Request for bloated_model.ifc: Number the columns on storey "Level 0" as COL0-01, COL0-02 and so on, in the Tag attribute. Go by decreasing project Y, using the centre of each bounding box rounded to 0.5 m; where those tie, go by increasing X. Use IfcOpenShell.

First a look at what the model holds.

```python
import ifcopenshell
import ifcopenshell.util.element
import ifcopenshell.util.placement

model = ifcopenshell.open("bloated_model.ifc")
print(model.schema)
storey = next(s for s in model.by_type("IfcBuildingStorey") if s.Name == "Level 0")
columns = [e for e in ifcopenshell.util.element.get_decomposition(storey) if e.is_a("IfcColumn")]
for e in sorted(columns, key=lambda e: e.id()):
    origin = ifcopenshell.util.placement.get_local_placement(e.ObjectPlacement)[:3, 3]
    print(e.id(), e.Tag, e.Name, origin.round(2) + 0.0, sep=" | ")
```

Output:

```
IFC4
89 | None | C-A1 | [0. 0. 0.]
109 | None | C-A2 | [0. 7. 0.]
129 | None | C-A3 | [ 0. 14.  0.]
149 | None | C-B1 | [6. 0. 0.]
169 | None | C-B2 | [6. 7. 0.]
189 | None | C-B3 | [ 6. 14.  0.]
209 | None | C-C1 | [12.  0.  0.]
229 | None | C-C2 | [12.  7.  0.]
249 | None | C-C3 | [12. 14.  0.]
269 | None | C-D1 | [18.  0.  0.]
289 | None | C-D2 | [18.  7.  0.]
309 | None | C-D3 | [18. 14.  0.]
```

```python
import ifcopenshell
import ifcopenshell.geom
import ifcopenshell.util.element
import ifcopenshell.util.shape

model = ifcopenshell.open("bloated_model.ifc")
settings = ifcopenshell.geom.settings()
settings.set("use-world-coords", True)


def centre(element):
    shape = ifcopenshell.geom.create_shape(settings, element)
    return ifcopenshell.util.shape.get_bbox_centroid(shape.geometry)


storey = next(s for s in model.by_type("IfcBuildingStorey") if s.Name == "Level 0")
columns = [e for e in ifcopenshell.util.element.get_decomposition(storey) if e.is_a("IfcColumn")]

# Insertion points can sit at a corner or the storey origin, so sort by the geometry (in metres).
centres = {e: centre(e) for e in columns}
columns.sort(key=lambda e: (-round(centres[e][1] / 0.5), centres[e][0]))

for i, e in enumerate(columns, start=1):
    number = f"COL0-{i:02d}"
    e.Tag = number
    print(e.id(), number)

model.write("bloated_model_edited.ifc")
```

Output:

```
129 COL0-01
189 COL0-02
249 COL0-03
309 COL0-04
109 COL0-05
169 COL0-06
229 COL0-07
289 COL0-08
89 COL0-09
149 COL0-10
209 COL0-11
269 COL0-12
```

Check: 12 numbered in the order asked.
